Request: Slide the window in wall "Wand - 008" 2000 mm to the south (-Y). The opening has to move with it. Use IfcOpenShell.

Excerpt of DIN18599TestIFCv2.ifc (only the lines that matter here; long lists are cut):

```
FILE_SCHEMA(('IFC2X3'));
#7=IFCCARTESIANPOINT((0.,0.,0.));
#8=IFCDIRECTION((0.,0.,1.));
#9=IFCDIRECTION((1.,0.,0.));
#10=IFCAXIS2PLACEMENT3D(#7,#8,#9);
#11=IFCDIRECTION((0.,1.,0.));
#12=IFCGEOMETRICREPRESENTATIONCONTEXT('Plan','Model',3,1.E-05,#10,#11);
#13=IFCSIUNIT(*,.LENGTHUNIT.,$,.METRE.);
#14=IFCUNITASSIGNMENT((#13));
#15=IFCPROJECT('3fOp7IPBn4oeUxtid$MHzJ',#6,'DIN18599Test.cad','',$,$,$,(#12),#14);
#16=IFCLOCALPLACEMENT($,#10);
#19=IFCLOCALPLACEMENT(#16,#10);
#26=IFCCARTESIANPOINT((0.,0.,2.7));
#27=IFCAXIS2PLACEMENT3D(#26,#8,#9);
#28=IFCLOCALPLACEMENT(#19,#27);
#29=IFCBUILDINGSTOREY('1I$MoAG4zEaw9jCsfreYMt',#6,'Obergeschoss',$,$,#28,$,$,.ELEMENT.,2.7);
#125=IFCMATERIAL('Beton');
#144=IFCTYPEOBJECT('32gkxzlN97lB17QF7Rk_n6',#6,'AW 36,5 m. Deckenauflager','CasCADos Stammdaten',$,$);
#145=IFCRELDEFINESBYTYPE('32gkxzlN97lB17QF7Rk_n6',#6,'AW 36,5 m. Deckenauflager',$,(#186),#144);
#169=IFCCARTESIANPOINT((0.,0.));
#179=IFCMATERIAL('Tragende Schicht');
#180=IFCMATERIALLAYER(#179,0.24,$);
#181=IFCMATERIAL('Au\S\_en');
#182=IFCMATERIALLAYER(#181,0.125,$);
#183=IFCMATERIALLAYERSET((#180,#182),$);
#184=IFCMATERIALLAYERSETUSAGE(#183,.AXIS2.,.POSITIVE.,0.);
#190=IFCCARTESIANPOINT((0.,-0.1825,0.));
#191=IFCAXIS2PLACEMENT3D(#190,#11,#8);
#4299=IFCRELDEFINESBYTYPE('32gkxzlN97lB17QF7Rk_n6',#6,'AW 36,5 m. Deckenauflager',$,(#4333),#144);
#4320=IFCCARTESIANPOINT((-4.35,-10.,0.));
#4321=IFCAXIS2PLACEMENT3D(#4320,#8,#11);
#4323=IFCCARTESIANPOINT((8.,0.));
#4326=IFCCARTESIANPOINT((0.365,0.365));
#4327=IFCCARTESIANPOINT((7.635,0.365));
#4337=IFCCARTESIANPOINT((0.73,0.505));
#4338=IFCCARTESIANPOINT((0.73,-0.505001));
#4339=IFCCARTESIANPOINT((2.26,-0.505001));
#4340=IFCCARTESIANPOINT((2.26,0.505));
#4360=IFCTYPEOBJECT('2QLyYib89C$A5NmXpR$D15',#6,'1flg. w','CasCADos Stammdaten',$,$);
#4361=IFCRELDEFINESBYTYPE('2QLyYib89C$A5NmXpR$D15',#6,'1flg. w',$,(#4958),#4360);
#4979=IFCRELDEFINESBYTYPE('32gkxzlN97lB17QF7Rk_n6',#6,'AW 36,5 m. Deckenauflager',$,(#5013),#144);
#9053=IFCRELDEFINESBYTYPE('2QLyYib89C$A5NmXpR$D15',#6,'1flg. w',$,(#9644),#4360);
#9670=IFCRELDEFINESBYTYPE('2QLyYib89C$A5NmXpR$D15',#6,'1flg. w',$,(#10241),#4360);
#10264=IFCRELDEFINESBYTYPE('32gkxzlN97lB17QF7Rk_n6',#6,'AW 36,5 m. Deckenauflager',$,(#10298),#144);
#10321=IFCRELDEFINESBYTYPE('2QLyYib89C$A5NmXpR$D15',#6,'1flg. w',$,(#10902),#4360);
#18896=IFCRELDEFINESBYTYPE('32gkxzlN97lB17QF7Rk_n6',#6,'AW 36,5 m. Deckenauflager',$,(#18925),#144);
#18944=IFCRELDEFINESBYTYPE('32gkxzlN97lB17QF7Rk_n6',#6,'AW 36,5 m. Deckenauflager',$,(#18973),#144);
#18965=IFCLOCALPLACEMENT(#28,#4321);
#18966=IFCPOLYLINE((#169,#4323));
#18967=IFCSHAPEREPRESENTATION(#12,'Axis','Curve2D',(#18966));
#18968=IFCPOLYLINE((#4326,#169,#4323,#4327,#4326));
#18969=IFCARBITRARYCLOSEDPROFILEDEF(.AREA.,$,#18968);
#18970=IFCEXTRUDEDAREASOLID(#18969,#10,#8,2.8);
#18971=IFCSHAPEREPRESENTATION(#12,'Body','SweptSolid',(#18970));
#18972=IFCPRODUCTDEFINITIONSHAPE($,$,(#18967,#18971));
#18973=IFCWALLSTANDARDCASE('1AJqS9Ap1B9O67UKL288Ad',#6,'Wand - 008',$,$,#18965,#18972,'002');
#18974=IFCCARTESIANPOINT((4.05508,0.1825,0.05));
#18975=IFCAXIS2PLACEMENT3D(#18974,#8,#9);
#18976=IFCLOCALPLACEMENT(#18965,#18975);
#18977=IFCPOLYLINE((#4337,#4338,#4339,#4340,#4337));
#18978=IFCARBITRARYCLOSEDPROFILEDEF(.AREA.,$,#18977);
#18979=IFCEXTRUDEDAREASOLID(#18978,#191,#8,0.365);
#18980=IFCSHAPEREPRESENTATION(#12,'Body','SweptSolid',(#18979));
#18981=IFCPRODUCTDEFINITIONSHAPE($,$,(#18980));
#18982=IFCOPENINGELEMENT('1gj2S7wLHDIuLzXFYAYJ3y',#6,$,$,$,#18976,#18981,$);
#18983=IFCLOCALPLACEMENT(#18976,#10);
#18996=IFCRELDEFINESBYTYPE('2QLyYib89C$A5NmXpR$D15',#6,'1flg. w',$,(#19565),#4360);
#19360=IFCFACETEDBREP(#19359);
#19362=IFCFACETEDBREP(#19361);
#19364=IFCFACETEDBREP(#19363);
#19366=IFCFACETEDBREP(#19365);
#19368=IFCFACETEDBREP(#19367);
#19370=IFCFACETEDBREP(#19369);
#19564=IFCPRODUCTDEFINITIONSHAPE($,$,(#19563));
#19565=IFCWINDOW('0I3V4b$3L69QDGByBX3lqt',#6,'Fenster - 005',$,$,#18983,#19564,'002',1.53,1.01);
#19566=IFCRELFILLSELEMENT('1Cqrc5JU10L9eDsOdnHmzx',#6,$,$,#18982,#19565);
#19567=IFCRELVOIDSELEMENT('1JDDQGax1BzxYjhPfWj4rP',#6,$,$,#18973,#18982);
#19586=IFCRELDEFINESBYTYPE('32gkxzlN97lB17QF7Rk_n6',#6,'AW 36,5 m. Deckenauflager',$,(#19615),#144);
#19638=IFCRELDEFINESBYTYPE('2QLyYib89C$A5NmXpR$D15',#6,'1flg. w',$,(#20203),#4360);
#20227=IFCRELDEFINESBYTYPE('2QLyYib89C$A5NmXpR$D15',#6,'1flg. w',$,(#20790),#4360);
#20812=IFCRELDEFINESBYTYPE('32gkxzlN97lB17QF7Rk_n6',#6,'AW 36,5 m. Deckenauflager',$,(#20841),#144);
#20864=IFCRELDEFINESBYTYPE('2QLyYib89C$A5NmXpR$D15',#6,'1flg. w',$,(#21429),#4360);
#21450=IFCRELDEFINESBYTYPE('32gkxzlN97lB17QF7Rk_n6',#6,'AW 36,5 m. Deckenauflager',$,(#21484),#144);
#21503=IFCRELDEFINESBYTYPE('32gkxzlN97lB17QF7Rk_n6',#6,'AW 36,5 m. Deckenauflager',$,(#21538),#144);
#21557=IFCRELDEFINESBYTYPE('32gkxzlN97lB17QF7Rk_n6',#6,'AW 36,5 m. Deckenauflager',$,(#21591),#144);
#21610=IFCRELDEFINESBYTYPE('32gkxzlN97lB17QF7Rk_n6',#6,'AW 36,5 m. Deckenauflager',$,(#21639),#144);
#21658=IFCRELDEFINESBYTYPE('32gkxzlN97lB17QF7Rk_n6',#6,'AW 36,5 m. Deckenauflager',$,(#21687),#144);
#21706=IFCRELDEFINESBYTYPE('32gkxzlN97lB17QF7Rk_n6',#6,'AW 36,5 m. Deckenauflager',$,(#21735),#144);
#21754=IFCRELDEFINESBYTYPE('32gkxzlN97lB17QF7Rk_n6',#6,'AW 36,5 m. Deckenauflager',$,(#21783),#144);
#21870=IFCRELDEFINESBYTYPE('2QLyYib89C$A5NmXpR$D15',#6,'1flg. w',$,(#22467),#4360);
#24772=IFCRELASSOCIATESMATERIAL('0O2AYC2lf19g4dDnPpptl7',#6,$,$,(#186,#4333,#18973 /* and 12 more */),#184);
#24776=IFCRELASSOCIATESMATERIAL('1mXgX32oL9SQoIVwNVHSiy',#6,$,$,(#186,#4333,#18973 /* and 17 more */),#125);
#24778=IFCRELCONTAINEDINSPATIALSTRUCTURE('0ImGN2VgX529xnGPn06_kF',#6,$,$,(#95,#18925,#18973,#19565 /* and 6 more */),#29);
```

```python
import ifcopenshell
import ifcopenshell.api.geometry
import ifcopenshell.util.placement
import ifcopenshell.util.unit

model = ifcopenshell.open("DIN18599TestIFCv2.ifc")
unit_scale = ifcopenshell.util.unit.calculate_unit_scale(model)

window = model.by_guid("0I3V4b$3L69QDGByBX3lqt")
opening = window.FillsVoids[0].RelatingOpeningElement
wall = opening.VoidsElements[0].RelatingBuildingElement

wall_matrix = ifcopenshell.util.placement.get_local_placement(wall.ObjectPlacement)
shift = wall_matrix[:3, 0] * -2 / unit_scale
before = ifcopenshell.util.placement.get_local_placement(window.ObjectPlacement)[:3, 3].copy()

# The window is placed relative to its opening, so it follows when the opening moves.
matrix = ifcopenshell.util.placement.get_local_placement(opening.ObjectPlacement)
matrix[:3, 3] += shift
ifcopenshell.api.geometry.edit_object_placement(
    model, product=opening, matrix=matrix, is_si=False, should_transform_children=True
)

after = ifcopenshell.util.placement.get_local_placement(window.ObjectPlacement)[:3, 3]
print("window moved by", (after - before).round(3) + 0.0)

model.write("DIN18599TestIFCv2_v2.ifc")
```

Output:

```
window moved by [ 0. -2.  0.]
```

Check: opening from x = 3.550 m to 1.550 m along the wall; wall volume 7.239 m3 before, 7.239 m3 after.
